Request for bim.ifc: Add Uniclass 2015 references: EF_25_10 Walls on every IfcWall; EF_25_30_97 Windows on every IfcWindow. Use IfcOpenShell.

First a look at what the model holds.

```python
import ifcopenshell

model = ifcopenshell.open("bim.ifc")
print(model.schema)
print("classifications:", [c.Name for c in model.by_type("IfcClassification")])
for ifc_class in ("IfcDoor", "IfcRoof", "IfcStair", "IfcWall", "IfcWindow"):
    print(ifc_class, len(model.by_type(ifc_class)))
```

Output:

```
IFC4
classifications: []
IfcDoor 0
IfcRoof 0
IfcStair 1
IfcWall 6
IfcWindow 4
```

```python
import ifcopenshell
import ifcopenshell.api.classification

model = ifcopenshell.open("bim.ifc")

system = ifcopenshell.api.classification.add_classification(model, classification="Uniclass 2015")

codes = {
    "IfcWall": ("EF_25_10", "Walls"),
    "IfcWindow": ("EF_25_30_97", "Windows"),
}
for ifc_class, (code, name) in codes.items():
    products = model.by_type(ifc_class)
    ifcopenshell.api.classification.add_reference(
        model, products=products, classification=system, identification=code, name=name
    )
    print(code, len(products))

model.write("bim-out.ifc")
```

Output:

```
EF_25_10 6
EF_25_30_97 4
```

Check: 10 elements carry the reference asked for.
